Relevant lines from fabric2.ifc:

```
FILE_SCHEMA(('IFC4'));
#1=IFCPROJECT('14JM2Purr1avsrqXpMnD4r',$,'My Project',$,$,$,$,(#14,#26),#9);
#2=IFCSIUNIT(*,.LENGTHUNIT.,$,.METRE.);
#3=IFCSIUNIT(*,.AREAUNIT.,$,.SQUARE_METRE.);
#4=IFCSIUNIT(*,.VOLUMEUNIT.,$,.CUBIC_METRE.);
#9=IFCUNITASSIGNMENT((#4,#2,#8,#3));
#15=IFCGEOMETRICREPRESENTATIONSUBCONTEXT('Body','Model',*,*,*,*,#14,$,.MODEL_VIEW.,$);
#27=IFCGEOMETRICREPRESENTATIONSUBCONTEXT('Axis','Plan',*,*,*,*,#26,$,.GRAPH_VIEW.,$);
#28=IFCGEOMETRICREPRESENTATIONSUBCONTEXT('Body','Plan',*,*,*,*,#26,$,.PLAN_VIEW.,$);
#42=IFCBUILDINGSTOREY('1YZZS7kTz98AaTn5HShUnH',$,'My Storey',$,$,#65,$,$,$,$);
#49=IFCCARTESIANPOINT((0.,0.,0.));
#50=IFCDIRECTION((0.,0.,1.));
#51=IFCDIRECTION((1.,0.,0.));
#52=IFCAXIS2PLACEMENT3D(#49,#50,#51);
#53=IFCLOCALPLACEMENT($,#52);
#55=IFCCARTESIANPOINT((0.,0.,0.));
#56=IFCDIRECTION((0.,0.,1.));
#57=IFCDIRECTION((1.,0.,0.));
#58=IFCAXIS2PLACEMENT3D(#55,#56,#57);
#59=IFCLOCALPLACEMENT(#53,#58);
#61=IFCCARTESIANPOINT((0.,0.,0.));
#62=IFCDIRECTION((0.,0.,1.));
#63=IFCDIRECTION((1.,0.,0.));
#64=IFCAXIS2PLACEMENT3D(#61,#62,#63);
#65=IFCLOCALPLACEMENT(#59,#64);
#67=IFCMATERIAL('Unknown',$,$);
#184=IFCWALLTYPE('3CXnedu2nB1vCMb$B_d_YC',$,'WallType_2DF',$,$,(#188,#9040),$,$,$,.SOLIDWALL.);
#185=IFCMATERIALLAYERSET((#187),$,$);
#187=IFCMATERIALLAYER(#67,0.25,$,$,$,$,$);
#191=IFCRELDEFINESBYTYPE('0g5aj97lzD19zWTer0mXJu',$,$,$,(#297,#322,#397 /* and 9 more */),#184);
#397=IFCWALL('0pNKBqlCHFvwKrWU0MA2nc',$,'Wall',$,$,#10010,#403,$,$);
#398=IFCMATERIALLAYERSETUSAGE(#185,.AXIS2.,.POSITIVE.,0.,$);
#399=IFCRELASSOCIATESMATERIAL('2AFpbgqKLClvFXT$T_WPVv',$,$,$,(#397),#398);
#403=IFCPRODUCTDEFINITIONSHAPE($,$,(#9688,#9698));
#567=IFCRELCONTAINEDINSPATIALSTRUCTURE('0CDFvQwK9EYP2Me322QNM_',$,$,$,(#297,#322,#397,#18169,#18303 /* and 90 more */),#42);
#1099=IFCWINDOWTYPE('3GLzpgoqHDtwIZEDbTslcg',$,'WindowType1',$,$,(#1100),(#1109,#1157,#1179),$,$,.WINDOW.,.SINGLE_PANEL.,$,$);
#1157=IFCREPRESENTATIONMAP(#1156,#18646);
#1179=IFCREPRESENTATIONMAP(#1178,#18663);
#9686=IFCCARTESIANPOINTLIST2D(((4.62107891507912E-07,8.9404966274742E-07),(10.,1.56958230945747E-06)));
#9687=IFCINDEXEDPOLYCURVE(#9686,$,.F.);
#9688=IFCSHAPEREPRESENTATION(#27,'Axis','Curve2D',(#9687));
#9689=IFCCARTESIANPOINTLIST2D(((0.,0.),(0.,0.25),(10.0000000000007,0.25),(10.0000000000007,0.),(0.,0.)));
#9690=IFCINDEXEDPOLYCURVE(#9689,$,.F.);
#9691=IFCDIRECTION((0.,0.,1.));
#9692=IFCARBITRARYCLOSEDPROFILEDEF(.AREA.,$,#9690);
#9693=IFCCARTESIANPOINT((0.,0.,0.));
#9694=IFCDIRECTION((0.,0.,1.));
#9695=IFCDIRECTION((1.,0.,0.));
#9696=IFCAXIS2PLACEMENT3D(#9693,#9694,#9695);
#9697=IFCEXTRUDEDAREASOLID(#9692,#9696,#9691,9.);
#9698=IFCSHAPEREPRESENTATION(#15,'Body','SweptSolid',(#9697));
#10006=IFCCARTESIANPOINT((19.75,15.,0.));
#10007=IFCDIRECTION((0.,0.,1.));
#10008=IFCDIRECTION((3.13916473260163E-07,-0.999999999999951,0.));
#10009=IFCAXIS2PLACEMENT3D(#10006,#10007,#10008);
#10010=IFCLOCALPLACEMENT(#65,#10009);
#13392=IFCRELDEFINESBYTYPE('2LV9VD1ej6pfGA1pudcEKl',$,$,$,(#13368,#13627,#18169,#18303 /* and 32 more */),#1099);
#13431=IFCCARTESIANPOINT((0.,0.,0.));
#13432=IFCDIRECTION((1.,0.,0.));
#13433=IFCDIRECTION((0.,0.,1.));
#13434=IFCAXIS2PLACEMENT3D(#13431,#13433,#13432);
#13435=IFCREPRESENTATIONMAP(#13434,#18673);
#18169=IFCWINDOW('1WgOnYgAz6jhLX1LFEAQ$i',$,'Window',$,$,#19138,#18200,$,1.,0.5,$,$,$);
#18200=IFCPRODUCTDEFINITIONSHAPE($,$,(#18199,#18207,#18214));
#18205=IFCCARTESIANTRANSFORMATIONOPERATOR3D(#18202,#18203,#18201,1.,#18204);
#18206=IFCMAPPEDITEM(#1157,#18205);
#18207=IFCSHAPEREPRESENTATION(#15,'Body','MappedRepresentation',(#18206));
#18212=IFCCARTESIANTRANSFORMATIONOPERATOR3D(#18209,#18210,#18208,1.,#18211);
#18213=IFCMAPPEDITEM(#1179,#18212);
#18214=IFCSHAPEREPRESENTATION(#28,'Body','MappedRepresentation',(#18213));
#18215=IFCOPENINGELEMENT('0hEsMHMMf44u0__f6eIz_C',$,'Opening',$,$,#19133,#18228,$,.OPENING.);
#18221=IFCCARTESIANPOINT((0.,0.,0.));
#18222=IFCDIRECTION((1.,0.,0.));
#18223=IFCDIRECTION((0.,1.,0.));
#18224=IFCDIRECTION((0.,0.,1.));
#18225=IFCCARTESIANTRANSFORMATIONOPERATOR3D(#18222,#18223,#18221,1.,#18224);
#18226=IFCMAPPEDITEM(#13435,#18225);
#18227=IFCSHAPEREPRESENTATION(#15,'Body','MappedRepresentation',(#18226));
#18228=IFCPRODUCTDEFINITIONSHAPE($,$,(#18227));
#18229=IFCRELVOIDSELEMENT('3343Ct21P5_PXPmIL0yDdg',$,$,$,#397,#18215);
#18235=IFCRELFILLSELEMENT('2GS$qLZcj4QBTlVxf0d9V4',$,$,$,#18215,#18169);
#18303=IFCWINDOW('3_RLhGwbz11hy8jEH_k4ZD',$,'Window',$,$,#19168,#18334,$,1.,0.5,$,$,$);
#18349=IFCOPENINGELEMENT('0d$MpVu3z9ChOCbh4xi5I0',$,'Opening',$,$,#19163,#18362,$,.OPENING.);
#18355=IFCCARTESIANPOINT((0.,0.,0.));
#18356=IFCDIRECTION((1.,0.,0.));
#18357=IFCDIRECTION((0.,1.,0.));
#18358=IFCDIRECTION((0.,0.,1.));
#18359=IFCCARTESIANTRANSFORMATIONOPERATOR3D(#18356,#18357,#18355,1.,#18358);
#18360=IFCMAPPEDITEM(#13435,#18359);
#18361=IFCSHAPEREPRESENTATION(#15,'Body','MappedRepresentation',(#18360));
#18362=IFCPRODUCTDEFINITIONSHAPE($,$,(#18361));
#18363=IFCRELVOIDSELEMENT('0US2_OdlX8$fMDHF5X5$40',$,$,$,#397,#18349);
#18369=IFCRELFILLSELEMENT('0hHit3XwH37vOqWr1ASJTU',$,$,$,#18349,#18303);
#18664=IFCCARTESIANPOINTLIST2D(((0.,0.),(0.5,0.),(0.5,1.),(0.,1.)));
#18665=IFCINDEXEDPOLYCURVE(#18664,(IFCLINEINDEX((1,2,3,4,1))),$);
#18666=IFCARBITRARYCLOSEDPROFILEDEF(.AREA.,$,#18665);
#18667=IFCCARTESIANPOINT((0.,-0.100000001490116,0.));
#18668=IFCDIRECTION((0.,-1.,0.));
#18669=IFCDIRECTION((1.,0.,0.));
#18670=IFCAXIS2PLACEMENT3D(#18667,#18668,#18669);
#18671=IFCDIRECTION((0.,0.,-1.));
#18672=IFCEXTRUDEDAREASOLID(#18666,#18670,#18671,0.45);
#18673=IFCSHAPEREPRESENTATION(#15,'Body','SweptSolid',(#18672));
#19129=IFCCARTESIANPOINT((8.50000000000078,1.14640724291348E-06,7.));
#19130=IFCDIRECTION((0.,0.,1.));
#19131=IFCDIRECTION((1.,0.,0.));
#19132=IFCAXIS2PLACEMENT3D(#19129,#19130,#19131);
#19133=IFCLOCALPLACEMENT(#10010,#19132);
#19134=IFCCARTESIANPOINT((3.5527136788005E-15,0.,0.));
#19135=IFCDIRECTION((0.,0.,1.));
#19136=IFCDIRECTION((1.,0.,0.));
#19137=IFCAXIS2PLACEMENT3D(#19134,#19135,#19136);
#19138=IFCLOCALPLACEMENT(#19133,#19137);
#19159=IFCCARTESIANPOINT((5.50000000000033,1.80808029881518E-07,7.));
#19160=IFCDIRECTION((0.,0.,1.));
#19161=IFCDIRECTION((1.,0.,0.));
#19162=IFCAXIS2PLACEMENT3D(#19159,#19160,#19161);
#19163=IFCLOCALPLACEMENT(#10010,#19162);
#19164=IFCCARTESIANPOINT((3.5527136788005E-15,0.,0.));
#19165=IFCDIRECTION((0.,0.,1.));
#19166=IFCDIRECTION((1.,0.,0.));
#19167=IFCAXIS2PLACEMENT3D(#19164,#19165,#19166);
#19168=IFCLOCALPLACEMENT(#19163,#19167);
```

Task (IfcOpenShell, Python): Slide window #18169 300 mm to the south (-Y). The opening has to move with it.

```python
import ifcopenshell
import ifcopenshell.api.geometry
import ifcopenshell.util.placement

model = ifcopenshell.open("fabric2.ifc")

window = model.by_guid("1WgOnYgAz6jhLX1LFEAQ$i")
opening = window.FillsVoids[0].RelatingOpeningElement
wall = opening.VoidsElements[0].RelatingBuildingElement

wall_matrix = ifcopenshell.util.placement.get_local_placement(wall.ObjectPlacement)
shift = wall_matrix[:3, 0] * 0.3
before = ifcopenshell.util.placement.get_local_placement(window.ObjectPlacement)[:3, 3].copy()

# The window is placed relative to its opening, so it follows when the opening moves.
matrix = ifcopenshell.util.placement.get_local_placement(opening.ObjectPlacement)
matrix[:3, 3] += shift
ifcopenshell.api.geometry.edit_object_placement(
    model, product=opening, matrix=matrix, is_si=False, should_transform_children=True
)

after = ifcopenshell.util.placement.get_local_placement(window.ObjectPlacement)[:3, 3]
print("window moved by", (after - before).round(3) + 0.0)

model.write("fabric2_updated.ifc")
```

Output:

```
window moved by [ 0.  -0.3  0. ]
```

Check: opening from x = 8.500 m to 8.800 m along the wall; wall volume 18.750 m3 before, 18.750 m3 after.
